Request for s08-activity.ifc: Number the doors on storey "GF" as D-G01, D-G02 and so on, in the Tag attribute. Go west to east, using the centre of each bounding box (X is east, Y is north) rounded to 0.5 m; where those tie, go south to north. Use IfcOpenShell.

First a look at what the model holds.

```python
import ifcopenshell
import ifcopenshell.util.element
import ifcopenshell.util.placement

model = ifcopenshell.open("s08-activity.ifc")
print(model.schema)
storey = next(s for s in model.by_type("IfcBuildingStorey") if s.Name == "GF")
doors = [e for e in ifcopenshell.util.element.get_decomposition(storey) if e.is_a("IfcDoor")]
for e in sorted(doors, key=lambda e: e.id()):
    origin = ifcopenshell.util.placement.get_local_placement(e.ObjectPlacement)[:3, 3]
    print(e.id(), e.Tag, e.Name, origin.round(2) + 0.0, sep=" | ")
```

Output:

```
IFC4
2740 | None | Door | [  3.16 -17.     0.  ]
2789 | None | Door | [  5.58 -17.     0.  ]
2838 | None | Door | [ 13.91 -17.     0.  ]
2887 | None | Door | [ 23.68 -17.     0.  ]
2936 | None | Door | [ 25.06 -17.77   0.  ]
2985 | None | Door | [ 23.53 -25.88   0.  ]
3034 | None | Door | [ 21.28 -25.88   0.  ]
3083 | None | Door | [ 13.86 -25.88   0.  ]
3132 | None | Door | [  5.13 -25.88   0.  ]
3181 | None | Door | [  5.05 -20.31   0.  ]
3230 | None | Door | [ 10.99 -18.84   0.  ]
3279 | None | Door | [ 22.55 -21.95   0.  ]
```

```python
import ifcopenshell
import ifcopenshell.geom
import ifcopenshell.util.element
import ifcopenshell.util.shape

model = ifcopenshell.open("s08-activity.ifc")
settings = ifcopenshell.geom.settings()
settings.set("use-world-coords", True)


def centre(element):
    shape = ifcopenshell.geom.create_shape(settings, element)
    return ifcopenshell.util.shape.get_bbox_centroid(shape.geometry)


storey = next(s for s in model.by_type("IfcBuildingStorey") if s.Name == "GF")
doors = [e for e in ifcopenshell.util.element.get_decomposition(storey) if e.is_a("IfcDoor")]

# Insertion points can sit at a corner or the storey origin, so sort by the geometry (in metres).
centres = {e: centre(e) for e in doors}
doors.sort(key=lambda e: (round(centres[e][0] / 0.5), centres[e][1]))

for i, e in enumerate(doors, start=1):
    number = f"D-G{i:02d}"
    e.Tag = number
    print(e.id(), number)

model.write("s08-activity_updated.ifc")
```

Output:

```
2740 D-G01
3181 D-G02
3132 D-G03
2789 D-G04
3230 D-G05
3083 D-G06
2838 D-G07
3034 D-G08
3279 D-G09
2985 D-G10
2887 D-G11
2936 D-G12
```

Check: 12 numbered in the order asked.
